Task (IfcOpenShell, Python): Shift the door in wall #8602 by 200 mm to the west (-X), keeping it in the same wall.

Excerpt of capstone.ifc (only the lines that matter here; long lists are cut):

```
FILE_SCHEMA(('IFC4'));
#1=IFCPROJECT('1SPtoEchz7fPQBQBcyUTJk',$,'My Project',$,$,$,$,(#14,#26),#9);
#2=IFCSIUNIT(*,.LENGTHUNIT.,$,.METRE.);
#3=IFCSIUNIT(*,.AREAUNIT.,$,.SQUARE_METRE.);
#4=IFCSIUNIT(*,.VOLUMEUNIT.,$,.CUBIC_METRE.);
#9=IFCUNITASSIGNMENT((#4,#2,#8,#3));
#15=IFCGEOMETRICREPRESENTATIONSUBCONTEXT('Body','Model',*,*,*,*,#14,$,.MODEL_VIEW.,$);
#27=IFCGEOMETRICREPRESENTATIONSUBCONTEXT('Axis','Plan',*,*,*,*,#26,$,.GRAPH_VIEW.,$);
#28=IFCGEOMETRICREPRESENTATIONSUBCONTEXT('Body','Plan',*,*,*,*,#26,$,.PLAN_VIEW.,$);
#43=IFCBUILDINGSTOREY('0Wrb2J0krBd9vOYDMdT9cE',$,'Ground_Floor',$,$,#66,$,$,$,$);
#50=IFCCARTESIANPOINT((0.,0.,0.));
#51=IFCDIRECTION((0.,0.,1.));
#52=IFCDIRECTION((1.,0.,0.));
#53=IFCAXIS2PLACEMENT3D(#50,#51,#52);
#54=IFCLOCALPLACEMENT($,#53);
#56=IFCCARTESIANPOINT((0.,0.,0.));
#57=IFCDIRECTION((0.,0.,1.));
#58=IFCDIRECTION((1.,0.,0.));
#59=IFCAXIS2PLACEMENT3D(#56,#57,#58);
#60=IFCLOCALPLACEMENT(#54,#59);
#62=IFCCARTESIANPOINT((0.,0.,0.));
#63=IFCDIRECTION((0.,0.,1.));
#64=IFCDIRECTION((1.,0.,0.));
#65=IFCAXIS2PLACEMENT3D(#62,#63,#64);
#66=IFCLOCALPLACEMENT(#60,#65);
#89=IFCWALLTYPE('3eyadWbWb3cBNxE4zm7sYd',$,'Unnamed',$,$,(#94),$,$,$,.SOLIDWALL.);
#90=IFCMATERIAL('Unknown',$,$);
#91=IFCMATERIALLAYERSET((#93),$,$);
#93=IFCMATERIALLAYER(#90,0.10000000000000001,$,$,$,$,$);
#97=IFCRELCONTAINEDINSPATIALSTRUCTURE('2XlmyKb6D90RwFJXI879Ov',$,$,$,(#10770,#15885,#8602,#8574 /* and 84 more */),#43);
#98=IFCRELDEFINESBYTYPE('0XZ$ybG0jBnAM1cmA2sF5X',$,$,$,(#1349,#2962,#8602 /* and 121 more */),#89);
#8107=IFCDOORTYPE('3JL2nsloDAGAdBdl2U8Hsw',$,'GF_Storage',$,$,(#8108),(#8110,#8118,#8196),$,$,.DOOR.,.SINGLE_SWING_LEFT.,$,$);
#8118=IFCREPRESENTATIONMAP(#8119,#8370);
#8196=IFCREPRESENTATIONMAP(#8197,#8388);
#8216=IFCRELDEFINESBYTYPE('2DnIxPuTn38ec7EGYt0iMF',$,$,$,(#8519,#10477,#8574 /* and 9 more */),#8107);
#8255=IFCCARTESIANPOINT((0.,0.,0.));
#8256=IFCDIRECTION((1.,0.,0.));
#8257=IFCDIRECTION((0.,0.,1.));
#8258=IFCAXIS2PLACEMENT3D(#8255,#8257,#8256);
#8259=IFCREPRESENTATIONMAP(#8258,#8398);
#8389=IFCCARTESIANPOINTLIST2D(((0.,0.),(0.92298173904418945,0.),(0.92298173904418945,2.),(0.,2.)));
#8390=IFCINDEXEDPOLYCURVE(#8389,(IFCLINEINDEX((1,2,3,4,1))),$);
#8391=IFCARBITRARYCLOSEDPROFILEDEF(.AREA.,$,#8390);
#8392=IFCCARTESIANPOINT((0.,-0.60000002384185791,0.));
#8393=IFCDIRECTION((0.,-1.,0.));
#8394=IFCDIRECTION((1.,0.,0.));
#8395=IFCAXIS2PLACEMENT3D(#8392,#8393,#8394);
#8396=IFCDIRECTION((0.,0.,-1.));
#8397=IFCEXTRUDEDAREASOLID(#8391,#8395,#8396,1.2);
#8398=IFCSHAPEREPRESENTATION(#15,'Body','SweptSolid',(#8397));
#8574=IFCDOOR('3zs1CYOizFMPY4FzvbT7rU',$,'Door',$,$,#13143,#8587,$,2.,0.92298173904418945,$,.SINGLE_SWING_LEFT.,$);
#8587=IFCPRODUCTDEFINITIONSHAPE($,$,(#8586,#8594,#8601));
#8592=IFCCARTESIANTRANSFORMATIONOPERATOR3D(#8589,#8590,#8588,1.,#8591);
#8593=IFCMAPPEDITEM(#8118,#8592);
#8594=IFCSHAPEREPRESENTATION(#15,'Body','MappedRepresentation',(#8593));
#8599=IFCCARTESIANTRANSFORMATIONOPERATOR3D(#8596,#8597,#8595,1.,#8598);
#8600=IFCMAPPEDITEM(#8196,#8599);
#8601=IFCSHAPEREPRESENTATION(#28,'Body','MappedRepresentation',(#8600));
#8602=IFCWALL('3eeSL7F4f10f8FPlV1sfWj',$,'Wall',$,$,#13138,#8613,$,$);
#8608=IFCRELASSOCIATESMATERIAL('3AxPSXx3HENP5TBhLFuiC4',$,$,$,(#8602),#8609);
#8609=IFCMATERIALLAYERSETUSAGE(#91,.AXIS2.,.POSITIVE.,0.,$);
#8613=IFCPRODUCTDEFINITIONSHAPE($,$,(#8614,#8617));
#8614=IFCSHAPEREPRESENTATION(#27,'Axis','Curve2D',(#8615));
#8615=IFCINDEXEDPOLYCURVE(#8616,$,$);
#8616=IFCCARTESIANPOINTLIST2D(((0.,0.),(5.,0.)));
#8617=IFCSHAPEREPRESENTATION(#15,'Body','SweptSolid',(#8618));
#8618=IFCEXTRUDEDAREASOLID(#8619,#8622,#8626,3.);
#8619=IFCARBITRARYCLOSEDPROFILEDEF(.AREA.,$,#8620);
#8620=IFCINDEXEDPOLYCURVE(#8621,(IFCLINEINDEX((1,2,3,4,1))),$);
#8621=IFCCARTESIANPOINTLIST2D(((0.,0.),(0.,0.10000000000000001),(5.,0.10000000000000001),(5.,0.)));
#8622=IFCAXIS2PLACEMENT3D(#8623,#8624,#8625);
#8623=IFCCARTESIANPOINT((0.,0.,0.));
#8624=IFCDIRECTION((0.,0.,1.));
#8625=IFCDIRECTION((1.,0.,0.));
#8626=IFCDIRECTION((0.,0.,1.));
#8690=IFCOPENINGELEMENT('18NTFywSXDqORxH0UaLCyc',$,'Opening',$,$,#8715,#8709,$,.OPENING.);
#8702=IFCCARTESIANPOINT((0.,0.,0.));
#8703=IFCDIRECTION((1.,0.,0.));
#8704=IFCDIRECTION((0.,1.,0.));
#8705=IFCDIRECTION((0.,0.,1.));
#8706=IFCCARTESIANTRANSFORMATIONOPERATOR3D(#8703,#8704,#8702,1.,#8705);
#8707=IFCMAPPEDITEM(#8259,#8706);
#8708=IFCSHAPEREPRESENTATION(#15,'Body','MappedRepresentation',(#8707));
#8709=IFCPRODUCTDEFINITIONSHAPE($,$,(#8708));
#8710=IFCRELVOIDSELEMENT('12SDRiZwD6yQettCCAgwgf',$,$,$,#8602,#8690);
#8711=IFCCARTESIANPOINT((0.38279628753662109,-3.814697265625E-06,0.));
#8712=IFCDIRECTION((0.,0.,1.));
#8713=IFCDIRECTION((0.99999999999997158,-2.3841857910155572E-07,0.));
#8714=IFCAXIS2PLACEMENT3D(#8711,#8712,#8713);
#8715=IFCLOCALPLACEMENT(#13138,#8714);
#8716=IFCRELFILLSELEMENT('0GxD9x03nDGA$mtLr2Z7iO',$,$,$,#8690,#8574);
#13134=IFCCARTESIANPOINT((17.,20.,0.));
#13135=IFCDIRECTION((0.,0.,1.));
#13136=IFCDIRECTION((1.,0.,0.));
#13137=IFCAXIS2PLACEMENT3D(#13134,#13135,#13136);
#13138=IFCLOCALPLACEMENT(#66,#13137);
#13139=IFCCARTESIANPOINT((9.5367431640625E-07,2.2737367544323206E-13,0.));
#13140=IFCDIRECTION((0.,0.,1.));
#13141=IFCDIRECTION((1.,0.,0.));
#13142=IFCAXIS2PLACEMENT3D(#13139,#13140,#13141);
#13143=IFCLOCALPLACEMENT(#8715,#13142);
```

```python
import ifcopenshell
import ifcopenshell.api.geometry
import ifcopenshell.util.placement
import ifcopenshell.util.unit

model = ifcopenshell.open("capstone.ifc")
unit_scale = ifcopenshell.util.unit.calculate_unit_scale(model)

door = model.by_id(8574)
opening = door.FillsVoids[0].RelatingOpeningElement
wall = opening.VoidsElements[0].RelatingBuildingElement

wall_matrix = ifcopenshell.util.placement.get_local_placement(wall.ObjectPlacement)
shift = wall_matrix[:3, 0] * -0.2 / unit_scale
before = ifcopenshell.util.placement.get_local_placement(door.ObjectPlacement)[:3, 3].copy()

# The door is placed relative to its opening, so it follows when the opening moves.
matrix = ifcopenshell.util.placement.get_local_placement(opening.ObjectPlacement)
matrix[:3, 3] += shift
ifcopenshell.api.geometry.edit_object_placement(
    model, product=opening, matrix=matrix, is_si=False, should_transform_children=True
)

after = ifcopenshell.util.placement.get_local_placement(door.ObjectPlacement)[:3, 3]
print("door moved by", (after - before).round(3) + 0.0)

model.write("capstone-out.ifc")
```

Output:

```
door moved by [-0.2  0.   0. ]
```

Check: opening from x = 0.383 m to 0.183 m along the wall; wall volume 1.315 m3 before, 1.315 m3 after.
